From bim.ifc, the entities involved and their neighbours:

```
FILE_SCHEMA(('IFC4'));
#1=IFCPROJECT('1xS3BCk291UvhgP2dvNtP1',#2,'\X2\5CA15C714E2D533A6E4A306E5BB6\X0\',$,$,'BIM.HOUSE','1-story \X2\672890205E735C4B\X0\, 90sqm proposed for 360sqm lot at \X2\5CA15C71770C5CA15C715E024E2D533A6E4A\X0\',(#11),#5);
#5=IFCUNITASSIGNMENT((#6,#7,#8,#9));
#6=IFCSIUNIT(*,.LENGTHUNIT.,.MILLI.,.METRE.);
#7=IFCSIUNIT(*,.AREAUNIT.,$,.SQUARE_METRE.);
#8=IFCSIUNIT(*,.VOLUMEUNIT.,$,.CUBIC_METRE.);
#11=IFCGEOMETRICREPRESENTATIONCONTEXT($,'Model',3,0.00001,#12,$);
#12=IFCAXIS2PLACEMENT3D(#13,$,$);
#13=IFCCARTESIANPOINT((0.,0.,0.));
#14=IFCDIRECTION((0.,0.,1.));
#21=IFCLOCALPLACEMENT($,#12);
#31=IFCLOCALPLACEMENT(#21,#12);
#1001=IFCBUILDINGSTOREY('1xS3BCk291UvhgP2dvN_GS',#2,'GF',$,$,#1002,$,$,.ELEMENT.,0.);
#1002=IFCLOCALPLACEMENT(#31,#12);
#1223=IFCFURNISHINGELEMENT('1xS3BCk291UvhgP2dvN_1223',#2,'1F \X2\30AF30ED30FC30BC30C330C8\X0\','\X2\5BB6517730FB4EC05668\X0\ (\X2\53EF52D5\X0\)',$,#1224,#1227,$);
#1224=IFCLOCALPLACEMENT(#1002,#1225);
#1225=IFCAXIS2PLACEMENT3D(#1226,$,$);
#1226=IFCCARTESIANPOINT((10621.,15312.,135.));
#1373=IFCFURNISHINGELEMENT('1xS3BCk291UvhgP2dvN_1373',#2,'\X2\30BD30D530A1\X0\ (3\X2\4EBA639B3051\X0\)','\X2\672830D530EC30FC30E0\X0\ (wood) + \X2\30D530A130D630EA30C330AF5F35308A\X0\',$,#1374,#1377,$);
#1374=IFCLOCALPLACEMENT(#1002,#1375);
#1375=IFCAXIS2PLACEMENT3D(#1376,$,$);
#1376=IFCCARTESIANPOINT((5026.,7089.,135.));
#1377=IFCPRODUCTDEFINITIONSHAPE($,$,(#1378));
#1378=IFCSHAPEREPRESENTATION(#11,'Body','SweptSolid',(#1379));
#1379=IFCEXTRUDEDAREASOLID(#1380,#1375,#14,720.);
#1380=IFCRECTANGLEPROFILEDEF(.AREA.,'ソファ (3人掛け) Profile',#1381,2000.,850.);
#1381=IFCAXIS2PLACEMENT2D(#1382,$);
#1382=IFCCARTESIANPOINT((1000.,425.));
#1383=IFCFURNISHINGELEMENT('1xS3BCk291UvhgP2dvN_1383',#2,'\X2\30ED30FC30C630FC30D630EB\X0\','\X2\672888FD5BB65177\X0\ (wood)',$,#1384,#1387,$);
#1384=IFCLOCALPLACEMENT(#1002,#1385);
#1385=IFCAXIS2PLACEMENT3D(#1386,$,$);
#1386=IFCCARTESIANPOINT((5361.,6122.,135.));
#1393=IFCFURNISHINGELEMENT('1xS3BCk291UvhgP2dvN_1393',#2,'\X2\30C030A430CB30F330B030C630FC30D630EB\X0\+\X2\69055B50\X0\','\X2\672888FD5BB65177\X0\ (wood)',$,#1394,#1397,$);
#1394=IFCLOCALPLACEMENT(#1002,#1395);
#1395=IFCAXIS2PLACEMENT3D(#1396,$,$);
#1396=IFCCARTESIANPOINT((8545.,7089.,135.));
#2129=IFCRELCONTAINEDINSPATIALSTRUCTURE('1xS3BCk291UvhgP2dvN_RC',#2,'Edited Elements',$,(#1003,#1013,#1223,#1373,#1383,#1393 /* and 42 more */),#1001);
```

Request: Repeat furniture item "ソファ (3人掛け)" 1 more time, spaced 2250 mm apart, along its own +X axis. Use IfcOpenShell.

```python
import ifcopenshell
import ifcopenshell.api.geometry
import ifcopenshell.api.root
import ifcopenshell.util.element
import ifcopenshell.util.placement

model = ifcopenshell.open("bim.ifc")


def reuse_history(source, copy):
    """copy_class also copies each property set's owner history, people and application; keep the originals."""
    for rel in copy.IsDefinedBy:
        if rel.is_a("IfcRelDefinesByProperties") and (history := rel.RelatingPropertyDefinition.OwnerHistory):
            rel.RelatingPropertyDefinition.OwnerHistory = source.OwnerHistory
            ifcopenshell.util.element.remove_deep2(model, history)


source = model.by_guid("1xS3BCk291UvhgP2dvN_1373")
base = ifcopenshell.util.placement.get_local_placement(source.ObjectPlacement)
step = base[:3, 0] * 2250.0

for i in range(1, 2):
    copy = ifcopenshell.api.root.copy_class(model, product=source)
    copy.Representation = ifcopenshell.util.element.copy_deep(
        model, source.Representation, exclude=["IfcGeometricRepresentationContext", "IfcRepresentationMap"]
    )
    reuse_history(source, copy)
    matrix = base.copy()
    matrix[:3, 3] += i * step
    print("added at", matrix[:3, 3].round(3) + 0.0)
    ifcopenshell.api.geometry.edit_object_placement(model, product=copy, matrix=matrix, is_si=False)

model.write("bim_rev.ifc")
```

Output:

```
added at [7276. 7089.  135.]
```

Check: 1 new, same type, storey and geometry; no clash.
